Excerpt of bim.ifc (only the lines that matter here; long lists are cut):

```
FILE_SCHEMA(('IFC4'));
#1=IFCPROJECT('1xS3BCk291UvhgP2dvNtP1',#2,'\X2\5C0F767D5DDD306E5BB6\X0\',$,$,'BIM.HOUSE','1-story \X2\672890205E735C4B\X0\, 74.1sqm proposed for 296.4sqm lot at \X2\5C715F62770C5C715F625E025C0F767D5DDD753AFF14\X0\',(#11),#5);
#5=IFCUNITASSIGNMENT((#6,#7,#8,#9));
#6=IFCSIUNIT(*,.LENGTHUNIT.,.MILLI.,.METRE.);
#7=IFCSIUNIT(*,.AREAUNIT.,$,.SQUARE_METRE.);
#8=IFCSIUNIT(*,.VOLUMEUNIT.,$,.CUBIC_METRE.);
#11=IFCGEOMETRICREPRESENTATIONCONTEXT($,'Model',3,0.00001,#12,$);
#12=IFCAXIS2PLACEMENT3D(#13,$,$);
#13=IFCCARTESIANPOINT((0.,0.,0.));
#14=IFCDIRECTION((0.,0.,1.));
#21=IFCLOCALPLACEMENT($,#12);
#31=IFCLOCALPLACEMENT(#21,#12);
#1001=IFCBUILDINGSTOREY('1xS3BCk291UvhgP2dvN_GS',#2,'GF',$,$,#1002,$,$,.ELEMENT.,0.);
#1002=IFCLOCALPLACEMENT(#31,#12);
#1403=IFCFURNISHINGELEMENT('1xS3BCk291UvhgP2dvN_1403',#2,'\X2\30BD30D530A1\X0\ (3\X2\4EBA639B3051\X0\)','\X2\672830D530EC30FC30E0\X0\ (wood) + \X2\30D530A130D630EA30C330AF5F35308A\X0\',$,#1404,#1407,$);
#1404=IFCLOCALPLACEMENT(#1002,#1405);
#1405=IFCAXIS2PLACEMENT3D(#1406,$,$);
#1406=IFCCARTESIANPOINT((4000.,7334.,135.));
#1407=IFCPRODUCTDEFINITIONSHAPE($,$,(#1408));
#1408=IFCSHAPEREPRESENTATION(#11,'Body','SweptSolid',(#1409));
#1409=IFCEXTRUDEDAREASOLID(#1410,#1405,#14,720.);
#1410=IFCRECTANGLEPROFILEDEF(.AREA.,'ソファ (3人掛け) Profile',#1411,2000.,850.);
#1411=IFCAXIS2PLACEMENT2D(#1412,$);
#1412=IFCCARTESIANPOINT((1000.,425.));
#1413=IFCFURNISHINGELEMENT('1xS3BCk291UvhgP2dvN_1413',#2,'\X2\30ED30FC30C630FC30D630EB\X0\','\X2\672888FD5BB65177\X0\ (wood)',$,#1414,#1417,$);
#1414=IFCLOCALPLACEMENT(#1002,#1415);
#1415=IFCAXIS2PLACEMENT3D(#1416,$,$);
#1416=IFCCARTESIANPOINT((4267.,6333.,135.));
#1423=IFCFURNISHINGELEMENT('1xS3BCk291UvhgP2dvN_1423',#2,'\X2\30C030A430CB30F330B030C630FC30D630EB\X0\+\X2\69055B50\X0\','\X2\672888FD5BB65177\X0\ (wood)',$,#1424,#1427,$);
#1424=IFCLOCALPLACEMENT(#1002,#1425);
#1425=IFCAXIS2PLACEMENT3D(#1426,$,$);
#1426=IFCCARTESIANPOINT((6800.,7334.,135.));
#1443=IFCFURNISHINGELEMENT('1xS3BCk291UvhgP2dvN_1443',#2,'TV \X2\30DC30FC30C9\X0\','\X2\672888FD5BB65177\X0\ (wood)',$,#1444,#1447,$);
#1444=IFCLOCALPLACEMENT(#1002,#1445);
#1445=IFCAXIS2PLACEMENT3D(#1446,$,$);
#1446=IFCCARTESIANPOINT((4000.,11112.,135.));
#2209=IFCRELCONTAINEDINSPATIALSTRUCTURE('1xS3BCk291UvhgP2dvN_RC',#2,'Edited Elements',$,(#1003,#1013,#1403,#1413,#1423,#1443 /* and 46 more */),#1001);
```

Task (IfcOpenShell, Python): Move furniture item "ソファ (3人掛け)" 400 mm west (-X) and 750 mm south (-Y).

```python
import ifcopenshell
import ifcopenshell.api.geometry
import ifcopenshell.util.placement
import ifcopenshell.util.unit

model = ifcopenshell.open("bim.ifc")
unit_scale = ifcopenshell.util.unit.calculate_unit_scale(model)

item = model.by_guid("1xS3BCk291UvhgP2dvN_1403")
matrix = ifcopenshell.util.placement.get_local_placement(item.ObjectPlacement)
matrix[0, 3] -= 0.4 / unit_scale
matrix[1, 3] -= 0.75 / unit_scale
ifcopenshell.api.geometry.edit_object_placement(model, product=item, matrix=matrix, is_si=False)

print(ifcopenshell.util.placement.get_local_placement(item.ObjectPlacement).round(3) + 0.0)

model.write("bim_updated.ifc")
```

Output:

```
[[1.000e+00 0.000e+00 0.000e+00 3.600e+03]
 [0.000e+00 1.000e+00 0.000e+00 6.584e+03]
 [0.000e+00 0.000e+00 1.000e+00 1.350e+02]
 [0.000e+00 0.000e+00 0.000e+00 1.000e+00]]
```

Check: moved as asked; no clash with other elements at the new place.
